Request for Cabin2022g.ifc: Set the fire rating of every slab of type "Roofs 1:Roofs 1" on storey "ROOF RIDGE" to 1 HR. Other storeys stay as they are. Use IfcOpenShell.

First a look at what the model holds.

```python
import ifcopenshell
import ifcopenshell.util.element

model = ifcopenshell.open("Cabin2022g.ifc")
print(model.schema)
storey = next(s for s in model.by_type("IfcBuildingStorey") if s.Name == "ROOF RIDGE")
slabs = [e for e in ifcopenshell.util.element.get_decomposition(storey) if e.is_a("IfcSlab")]
seen = {}
for e in slabs:
    element_type = ifcopenshell.util.element.get_type(e)
    key = (element_type.Name if element_type != e and element_type else None, ifcopenshell.util.element.get_pset(e, "Pset_SlabCommon", "FireRating"))
    seen[key] = seen.get(key, 0) + 1
for (name, value), count in sorted(seen.items(), key=str):
    print(count, "x", name, "|", value)
```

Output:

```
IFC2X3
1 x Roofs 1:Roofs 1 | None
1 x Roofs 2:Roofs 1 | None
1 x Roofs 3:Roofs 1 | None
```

```python
import ifcopenshell
import ifcopenshell.api.pset
import ifcopenshell.util.element

model = ifcopenshell.open("Cabin2022g.ifc")

storey = next(s for s in model.by_type("IfcBuildingStorey") if s.Name == "ROOF RIDGE")
slabs = [e for e in ifcopenshell.util.element.get_decomposition(storey) if e.is_a("IfcSlab")]

count = 0
for e in slabs:
    element_type = ifcopenshell.util.element.get_type(e)
    if element_type in (None, e) or element_type.Name != "Roofs 1:Roofs 1":
        continue
    # add_pset returns the element's existing set when there is one.
    pset = ifcopenshell.api.pset.add_pset(model, product=e, name="Pset_SlabCommon")
    ifcopenshell.api.pset.edit_pset(model, pset=pset, properties={"FireRating": "1 HR"})
    count += 1

print(count, "slabs updated")

model.write("Cabin2022g_v2.ifc")
```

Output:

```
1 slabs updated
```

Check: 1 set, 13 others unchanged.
